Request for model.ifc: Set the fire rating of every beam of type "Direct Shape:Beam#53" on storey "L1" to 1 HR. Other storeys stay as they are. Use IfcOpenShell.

First a look at what the model holds.

```python
import ifcopenshell
import ifcopenshell.util.element

model = ifcopenshell.open("model.ifc")
print(model.schema)
storey = next(s for s in model.by_type("IfcBuildingStorey") if s.Name == "L1")
beams = [e for e in ifcopenshell.util.element.get_decomposition(storey) if e.is_a("IfcBeam")]
seen = {}
for e in beams:
    element_type = ifcopenshell.util.element.get_type(e)
    key = (element_type.Name if element_type != e and element_type else None, ifcopenshell.util.element.get_pset(e, "Pset_BeamCommon", "FireRating"))
    seen[key] = seen.get(key, 0) + 1
for (name, value), count in sorted(seen.items(), key=str):
    print(count, "x", name, "|", value)
```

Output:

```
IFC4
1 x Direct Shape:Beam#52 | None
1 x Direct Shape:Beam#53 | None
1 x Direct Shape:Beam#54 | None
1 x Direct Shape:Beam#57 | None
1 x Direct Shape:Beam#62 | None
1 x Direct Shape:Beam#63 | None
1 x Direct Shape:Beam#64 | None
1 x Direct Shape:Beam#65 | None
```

```python
import ifcopenshell
import ifcopenshell.api.pset
import ifcopenshell.util.element

model = ifcopenshell.open("model.ifc")

storey = next(s for s in model.by_type("IfcBuildingStorey") if s.Name == "L1")
beams = [e for e in ifcopenshell.util.element.get_decomposition(storey) if e.is_a("IfcBeam")]

count = 0
for e in beams:
    element_type = ifcopenshell.util.element.get_type(e)
    if element_type in (None, e) or element_type.Name != "Direct Shape:Beam#53":
        continue
    # add_pset returns the element's existing set when there is one.
    pset = ifcopenshell.api.pset.add_pset(model, product=e, name="Pset_BeamCommon")
    ifcopenshell.api.pset.edit_pset(model, pset=pset, properties={"FireRating": "1 HR"})
    count += 1

print(count, "beams updated")

model.write("model-out.ifc")
```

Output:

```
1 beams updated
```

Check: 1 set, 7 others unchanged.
